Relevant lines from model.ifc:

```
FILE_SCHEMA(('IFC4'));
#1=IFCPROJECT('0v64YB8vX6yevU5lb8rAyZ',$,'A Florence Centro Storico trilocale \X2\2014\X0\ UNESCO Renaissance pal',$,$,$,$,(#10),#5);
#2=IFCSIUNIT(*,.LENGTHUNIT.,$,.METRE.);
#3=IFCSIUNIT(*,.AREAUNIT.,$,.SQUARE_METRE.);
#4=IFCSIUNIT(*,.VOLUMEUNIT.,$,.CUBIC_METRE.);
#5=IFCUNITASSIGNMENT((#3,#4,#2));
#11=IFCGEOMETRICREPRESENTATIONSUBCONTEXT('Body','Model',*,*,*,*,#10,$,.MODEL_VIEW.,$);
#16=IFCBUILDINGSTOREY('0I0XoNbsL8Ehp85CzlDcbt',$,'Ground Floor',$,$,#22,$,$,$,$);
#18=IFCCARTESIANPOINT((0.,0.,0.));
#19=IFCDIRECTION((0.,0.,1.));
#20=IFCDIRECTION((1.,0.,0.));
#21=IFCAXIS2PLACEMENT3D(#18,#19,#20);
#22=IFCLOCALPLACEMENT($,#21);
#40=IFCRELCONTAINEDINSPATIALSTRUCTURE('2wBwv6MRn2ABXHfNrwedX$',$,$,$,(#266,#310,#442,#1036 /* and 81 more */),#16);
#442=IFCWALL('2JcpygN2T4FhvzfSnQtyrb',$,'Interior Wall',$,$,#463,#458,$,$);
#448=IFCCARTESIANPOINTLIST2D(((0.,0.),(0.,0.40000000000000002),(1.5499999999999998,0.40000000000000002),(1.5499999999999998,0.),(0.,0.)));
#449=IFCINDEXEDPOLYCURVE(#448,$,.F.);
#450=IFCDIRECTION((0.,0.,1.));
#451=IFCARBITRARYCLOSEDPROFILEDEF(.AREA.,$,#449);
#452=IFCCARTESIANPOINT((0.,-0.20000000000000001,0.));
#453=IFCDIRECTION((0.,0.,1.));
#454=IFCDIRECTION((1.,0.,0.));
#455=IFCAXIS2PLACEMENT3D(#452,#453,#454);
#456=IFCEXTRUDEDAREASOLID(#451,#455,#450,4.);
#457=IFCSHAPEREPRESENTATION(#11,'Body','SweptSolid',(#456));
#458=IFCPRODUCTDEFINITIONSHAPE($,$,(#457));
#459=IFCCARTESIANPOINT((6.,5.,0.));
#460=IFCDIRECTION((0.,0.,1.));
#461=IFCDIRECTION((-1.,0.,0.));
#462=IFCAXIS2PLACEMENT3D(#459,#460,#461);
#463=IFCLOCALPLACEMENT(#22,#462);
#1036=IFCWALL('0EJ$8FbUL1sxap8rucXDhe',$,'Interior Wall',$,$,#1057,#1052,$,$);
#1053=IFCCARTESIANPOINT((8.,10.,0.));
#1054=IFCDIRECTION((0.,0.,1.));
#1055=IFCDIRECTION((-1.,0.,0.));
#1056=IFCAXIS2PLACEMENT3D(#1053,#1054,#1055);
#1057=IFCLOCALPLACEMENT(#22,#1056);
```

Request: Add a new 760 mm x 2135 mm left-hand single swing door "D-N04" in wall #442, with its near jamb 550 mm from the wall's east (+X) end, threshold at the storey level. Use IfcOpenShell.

```python
import numpy as np
import ifcopenshell
import ifcopenshell.api.feature
import ifcopenshell.api.geometry
import ifcopenshell.api.root
import ifcopenshell.api.spatial
import ifcopenshell.geom
import ifcopenshell.util.element
import ifcopenshell.util.placement
import ifcopenshell.util.representation
import ifcopenshell.util.shape
import ifcopenshell.util.unit

model = ifcopenshell.open("model.ifc")
unit_scale = ifcopenshell.util.unit.calculate_unit_scale(model)
settings = ifcopenshell.geom.settings()


def volume(element):
    """Net volume in cubic metres, openings subtracted."""
    shape = ifcopenshell.geom.create_shape(settings, element)
    return ifcopenshell.util.shape.get_volume(shape.geometry)


wall = model.by_id(442)
storey = ifcopenshell.util.element.get_container(wall, ifc_class="IfcBuildingStorey")
context = ifcopenshell.util.representation.get_context(model, "Model", "Body", "MODEL_VIEW")
before = volume(wall)

width, height, from_end, sill = 0.76, 2.135, 0.55, 0.0  # metres

# The wall runs along its own X axis, and the end named is its -X end.
wall_shape = ifcopenshell.geom.create_shape(settings, wall)
x, y, z = ifcopenshell.util.shape.get_vertices(wall_shape.geometry).T
start = x.min() + from_end
face, thickness = float(y.min()), float(y.max() - y.min())
wall_matrix = ifcopenshell.util.placement.get_local_placement(wall.ObjectPlacement)
level = ifcopenshell.util.placement.get_local_placement(storey.ObjectPlacement)[2, 3]


def in_wall(x, y):
    """Placement at x, y metres in the wall's axes, at sill height."""
    matrix = wall_matrix.copy()
    matrix[:, 3] = wall_matrix @ np.array([x / unit_scale, y / unit_scale, 0.0, 1.0])
    matrix[2, 3] = level + sill / unit_scale
    return matrix


# Opening: a box that overshoots both wall faces by 50 mm.
opening = ifcopenshell.api.root.create_entity(model, ifc_class="IfcOpeningElement", predefined_type="OPENING")
box = ifcopenshell.api.geometry.add_wall_representation(
    model, context=context, length=width, height=height, thickness=thickness + 0.1
)
ifcopenshell.api.geometry.assign_representation(model, product=opening, representation=box)
ifcopenshell.api.geometry.edit_object_placement(model, product=opening, matrix=in_wall(start, face - 0.05), is_si=False)
ifcopenshell.api.feature.add_feature(model, feature=opening, element=wall)

door = ifcopenshell.api.root.create_entity(model, ifc_class="IfcDoor", name="D-N04", predefined_type="DOOR")
door.OverallWidth, door.OverallHeight = width / unit_scale, height / unit_scale
door.OperationType = "SINGLE_SWING_LEFT"
body = ifcopenshell.api.geometry.add_door_representation(
    model,
    context=context,
    overall_width=door.OverallWidth,
    overall_height=door.OverallHeight,
    operation_type="SINGLE_SWING_LEFT",
    lining_properties={"LiningDepth": thickness / unit_scale, "ThresholdDepth": thickness / unit_scale},
)
ifcopenshell.api.geometry.assign_representation(model, product=door, representation=body)
ifcopenshell.api.spatial.assign_container(model, products=[door], relating_structure=storey)
ifcopenshell.api.feature.add_filling(model, opening=opening, element=door)

# The lining spans the wall, so the door starts at the wall face.
ifcopenshell.api.geometry.edit_object_placement(model, product=door, matrix=in_wall(start, face), is_si=False)

after = volume(wall)

print(f"wall volume {before:.3f} -> {after:.3f} m3")

model.write("model-out.ifc")
```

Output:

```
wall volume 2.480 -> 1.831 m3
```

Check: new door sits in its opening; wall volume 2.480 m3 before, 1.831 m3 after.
